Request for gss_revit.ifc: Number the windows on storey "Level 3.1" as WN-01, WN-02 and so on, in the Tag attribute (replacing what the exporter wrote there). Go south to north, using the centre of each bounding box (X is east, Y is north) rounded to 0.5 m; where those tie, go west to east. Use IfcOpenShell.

First a look at what the model holds.

```python
import ifcopenshell
import ifcopenshell.util.element
import ifcopenshell.util.placement

model = ifcopenshell.open("gss_revit.ifc")
print(model.schema)
storey = next(s for s in model.by_type("IfcBuildingStorey") if s.Name == "Level 3.1")
windows = [e for e in ifcopenshell.util.element.get_decomposition(storey) if e.is_a("IfcWindow")]
for e in sorted(windows, key=lambda e: e.id()):
    origin = ifcopenshell.util.placement.get_local_placement(e.ObjectPlacement)[:3, 3]
    print(e.id(), e.Tag, e.Name, origin.round(2) + 0.0, sep=" | ")
```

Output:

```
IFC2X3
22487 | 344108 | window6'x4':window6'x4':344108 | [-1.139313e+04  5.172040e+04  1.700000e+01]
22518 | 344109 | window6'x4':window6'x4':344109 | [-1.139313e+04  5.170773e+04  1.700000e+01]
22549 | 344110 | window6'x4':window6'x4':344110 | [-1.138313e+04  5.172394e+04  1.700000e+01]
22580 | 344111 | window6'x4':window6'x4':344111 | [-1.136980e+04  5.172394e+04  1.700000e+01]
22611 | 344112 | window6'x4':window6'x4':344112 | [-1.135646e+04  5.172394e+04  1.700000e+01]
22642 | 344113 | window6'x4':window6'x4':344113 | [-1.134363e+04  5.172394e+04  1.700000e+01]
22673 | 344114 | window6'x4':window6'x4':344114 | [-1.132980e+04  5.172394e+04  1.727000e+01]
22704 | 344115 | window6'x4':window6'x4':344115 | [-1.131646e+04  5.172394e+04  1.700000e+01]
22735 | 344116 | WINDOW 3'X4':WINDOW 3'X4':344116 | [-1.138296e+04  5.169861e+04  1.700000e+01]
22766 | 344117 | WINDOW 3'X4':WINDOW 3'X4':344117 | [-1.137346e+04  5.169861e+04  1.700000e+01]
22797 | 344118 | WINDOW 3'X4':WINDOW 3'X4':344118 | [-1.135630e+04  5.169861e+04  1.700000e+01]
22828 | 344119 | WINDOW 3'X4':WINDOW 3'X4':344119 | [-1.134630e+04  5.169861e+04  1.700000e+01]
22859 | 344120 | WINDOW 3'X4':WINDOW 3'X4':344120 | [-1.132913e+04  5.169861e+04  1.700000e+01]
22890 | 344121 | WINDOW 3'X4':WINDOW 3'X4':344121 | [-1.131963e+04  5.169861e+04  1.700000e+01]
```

```python
import ifcopenshell
import ifcopenshell.geom
import ifcopenshell.util.element
import ifcopenshell.util.shape

model = ifcopenshell.open("gss_revit.ifc")
settings = ifcopenshell.geom.settings()
settings.set("use-world-coords", True)


def centre(element):
    shape = ifcopenshell.geom.create_shape(settings, element)
    return ifcopenshell.util.shape.get_bbox_centroid(shape.geometry)


storey = next(s for s in model.by_type("IfcBuildingStorey") if s.Name == "Level 3.1")
windows = [e for e in ifcopenshell.util.element.get_decomposition(storey) if e.is_a("IfcWindow")]

# Insertion points can sit at a corner or the storey origin, so sort by the geometry (in metres).
centres = {e: centre(e) for e in windows}
windows.sort(key=lambda e: (round(centres[e][1] / 0.5), centres[e][0]))

for i, e in enumerate(windows, start=1):
    number = f"WN-{i:02d}"
    e.Tag = number
    print(e.id(), number)

model.write("gss_revit-out.ifc")
```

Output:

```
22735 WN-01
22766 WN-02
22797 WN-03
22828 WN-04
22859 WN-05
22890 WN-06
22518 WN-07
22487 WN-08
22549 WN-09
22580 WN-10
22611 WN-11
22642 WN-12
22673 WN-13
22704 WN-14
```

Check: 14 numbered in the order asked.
